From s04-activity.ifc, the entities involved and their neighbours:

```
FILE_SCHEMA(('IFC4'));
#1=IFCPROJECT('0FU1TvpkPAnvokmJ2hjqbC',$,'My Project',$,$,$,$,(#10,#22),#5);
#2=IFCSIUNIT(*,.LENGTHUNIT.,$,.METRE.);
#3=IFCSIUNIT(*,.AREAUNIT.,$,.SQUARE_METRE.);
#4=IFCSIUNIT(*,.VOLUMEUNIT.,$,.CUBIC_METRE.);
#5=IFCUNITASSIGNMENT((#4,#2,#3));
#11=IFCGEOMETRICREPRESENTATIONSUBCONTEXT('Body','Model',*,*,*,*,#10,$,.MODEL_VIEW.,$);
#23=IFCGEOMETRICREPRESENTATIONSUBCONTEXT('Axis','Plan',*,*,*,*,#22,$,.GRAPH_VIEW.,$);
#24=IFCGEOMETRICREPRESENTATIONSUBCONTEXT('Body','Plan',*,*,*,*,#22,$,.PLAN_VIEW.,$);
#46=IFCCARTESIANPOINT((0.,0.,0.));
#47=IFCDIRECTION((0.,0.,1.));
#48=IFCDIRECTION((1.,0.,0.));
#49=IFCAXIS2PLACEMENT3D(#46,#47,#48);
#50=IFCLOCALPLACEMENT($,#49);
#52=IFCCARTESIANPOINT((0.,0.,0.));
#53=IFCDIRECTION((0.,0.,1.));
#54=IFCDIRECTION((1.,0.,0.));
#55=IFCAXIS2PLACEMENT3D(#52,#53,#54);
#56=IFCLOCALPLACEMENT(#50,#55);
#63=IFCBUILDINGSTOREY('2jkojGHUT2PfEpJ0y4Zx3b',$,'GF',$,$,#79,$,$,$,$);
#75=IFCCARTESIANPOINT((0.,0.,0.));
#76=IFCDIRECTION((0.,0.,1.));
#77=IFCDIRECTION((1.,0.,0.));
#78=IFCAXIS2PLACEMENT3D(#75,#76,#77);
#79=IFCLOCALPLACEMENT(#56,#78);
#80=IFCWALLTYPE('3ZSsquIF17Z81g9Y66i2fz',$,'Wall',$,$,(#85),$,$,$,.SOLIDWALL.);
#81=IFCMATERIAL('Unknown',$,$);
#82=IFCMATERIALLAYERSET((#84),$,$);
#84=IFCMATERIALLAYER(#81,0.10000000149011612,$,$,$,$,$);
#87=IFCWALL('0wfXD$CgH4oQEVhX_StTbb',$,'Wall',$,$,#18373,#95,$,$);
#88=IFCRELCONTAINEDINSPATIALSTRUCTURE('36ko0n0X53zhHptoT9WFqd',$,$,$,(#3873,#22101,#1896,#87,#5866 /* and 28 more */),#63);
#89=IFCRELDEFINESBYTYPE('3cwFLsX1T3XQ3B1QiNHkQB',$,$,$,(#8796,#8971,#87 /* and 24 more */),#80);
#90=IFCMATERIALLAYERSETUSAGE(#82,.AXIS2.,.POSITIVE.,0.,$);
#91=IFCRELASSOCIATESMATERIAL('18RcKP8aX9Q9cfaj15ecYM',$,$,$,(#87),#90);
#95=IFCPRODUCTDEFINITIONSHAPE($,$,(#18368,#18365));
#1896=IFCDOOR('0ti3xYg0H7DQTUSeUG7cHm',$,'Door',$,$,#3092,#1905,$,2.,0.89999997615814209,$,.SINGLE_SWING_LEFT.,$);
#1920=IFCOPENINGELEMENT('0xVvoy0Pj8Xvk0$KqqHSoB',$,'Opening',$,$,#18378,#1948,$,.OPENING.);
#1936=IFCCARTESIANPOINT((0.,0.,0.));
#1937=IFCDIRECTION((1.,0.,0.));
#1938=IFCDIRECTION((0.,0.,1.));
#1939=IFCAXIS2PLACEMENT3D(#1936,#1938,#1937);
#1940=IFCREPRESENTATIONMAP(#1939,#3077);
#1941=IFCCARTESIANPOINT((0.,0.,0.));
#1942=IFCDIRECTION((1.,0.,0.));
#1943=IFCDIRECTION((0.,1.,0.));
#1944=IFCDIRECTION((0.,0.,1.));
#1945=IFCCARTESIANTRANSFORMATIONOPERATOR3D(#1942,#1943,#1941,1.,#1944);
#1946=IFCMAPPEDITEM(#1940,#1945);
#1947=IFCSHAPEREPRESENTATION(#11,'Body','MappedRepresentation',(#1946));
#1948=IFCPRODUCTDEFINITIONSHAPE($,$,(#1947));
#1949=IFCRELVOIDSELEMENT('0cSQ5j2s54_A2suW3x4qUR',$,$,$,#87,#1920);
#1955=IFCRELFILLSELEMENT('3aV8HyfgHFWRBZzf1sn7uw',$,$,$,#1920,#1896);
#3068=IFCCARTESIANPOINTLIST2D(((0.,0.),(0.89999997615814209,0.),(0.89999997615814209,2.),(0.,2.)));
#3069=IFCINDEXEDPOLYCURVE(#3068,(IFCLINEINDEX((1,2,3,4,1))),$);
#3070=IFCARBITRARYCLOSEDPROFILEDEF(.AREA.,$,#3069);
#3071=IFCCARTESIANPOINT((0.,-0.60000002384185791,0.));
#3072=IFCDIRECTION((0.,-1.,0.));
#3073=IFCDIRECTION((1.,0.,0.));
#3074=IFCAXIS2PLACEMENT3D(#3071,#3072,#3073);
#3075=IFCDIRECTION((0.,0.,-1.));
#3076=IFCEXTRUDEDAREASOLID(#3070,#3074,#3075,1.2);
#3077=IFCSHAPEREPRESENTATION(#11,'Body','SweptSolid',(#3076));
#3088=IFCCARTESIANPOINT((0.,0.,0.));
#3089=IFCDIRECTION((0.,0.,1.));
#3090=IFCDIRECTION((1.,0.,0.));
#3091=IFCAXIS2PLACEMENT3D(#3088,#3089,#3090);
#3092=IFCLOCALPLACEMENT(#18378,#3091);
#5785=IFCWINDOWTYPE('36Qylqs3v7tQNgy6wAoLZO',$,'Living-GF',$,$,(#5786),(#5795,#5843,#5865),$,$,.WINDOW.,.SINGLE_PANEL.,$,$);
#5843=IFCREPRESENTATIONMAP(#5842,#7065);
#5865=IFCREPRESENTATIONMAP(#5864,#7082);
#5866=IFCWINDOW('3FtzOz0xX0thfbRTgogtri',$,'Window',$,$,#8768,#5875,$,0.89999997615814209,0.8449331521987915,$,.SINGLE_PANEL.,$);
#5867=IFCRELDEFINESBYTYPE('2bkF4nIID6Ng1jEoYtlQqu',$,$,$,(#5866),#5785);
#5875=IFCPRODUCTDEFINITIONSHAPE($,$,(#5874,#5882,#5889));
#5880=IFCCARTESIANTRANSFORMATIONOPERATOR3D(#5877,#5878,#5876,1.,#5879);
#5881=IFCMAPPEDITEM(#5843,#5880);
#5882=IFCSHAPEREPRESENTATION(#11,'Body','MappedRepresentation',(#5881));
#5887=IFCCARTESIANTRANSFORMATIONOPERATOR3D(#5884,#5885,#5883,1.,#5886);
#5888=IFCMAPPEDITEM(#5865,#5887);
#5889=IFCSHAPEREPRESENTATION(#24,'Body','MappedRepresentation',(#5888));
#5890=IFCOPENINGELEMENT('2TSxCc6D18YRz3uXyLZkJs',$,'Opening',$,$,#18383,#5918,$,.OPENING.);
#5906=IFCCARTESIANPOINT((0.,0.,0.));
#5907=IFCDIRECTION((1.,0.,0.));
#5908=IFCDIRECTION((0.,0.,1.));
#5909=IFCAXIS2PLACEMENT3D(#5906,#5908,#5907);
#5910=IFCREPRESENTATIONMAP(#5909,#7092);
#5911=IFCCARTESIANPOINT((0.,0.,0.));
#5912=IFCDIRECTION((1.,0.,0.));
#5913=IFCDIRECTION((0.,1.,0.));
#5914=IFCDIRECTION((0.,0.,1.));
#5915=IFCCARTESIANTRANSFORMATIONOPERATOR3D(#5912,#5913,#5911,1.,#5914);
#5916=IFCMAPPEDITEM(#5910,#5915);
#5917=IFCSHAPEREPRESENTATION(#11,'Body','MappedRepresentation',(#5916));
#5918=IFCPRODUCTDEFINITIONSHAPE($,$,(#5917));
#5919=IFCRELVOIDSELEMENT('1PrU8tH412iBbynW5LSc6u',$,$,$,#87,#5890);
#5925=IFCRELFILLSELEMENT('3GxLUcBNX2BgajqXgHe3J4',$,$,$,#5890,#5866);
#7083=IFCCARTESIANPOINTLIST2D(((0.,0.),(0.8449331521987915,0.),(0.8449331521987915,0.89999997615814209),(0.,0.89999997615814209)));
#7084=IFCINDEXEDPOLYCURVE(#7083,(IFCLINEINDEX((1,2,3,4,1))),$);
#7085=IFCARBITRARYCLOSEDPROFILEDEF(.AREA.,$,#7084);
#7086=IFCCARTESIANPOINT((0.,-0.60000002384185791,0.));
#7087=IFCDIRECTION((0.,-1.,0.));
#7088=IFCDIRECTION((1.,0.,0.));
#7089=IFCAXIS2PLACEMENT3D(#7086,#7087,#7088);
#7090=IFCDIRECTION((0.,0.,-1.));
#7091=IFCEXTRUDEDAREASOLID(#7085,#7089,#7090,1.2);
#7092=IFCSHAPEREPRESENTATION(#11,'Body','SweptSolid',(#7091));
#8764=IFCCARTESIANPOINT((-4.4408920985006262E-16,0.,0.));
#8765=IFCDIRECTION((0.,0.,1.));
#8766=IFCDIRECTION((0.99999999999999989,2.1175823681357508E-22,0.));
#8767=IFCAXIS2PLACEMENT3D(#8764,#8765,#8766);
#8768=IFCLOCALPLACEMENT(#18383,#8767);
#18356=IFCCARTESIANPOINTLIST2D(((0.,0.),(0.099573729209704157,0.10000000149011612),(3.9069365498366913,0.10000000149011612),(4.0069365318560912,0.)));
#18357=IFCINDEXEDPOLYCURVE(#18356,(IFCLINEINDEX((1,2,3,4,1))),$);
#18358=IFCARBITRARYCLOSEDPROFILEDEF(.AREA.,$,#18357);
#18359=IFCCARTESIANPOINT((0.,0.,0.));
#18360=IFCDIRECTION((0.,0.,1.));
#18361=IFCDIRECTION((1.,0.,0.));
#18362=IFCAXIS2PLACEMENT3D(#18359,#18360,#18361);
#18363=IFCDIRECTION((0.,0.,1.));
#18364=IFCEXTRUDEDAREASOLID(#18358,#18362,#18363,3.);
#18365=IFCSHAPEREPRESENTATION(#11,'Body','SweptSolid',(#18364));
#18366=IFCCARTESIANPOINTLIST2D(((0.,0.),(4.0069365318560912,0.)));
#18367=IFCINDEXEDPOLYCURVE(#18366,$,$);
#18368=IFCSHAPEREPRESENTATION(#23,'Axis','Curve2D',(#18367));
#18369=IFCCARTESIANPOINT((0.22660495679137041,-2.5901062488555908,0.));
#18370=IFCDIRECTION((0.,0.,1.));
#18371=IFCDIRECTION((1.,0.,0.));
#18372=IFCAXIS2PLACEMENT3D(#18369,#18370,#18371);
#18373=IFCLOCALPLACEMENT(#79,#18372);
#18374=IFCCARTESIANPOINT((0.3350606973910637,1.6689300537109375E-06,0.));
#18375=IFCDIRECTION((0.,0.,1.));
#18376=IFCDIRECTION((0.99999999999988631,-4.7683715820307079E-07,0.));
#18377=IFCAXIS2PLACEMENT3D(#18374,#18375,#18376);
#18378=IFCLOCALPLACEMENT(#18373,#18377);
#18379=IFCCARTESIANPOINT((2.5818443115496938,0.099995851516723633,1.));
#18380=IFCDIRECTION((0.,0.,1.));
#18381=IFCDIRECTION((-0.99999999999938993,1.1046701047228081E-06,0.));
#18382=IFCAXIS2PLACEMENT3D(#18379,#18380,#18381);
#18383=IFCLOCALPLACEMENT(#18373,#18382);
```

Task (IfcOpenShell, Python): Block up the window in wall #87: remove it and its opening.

```python
import ifcopenshell
import ifcopenshell.api.feature
import ifcopenshell.api.root
import ifcopenshell.geom
import ifcopenshell.util.shape

model = ifcopenshell.open("s04-activity.ifc")
settings = ifcopenshell.geom.settings()


def volume(element):
    """Net volume in cubic metres, openings subtracted."""
    shape = ifcopenshell.geom.create_shape(settings, element)
    return ifcopenshell.util.shape.get_volume(shape.geometry)


window = model.by_guid("3FtzOz0xX0thfbRTgogtri")
opening = window.FillsVoids[0].RelatingOpeningElement
wall = opening.VoidsElements[0].RelatingBuildingElement
before = volume(wall)

ifcopenshell.api.root.remove_product(model, product=window)
ifcopenshell.api.feature.remove_feature(model, feature=opening)

after = volume(wall)

print(f"wall volume {before:.3f} -> {after:.3f} m3")

model.write("s04-activity_updated.ifc")
```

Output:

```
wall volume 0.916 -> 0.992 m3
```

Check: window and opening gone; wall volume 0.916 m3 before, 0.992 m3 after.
